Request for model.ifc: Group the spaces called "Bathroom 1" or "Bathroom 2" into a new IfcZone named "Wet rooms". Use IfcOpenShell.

First a look at what the model holds.

```python
import ifcopenshell

model = ifcopenshell.open("model.ifc")
print(model.schema)
seen = {}
for space in model.by_type("IfcSpace"):
    seen[space.LongName] = seen.get(space.LongName, 0) + 1
for name, count in sorted(seen.items(), key=str):
    print(count, "x", name)
print("zones:", [z.Name for z in model.by_type("IfcZone")][:20])
```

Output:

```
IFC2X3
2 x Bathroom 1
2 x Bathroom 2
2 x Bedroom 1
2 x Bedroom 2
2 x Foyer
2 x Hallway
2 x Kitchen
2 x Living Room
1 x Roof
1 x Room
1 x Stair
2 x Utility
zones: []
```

```python
import ifcopenshell
import ifcopenshell.api.group
import ifcopenshell.api.root

model = ifcopenshell.open("model.ifc")

names = {"Bathroom 1", "Bathroom 2"}
spaces = [s for s in model.by_type("IfcSpace") if s.LongName in names]

zone = ifcopenshell.api.root.create_entity(model, ifc_class="IfcZone", name="Wet rooms")
ifcopenshell.api.group.assign_group(model, products=spaces, group=zone)
print(len(spaces), "spaces in", zone.Name)

model.write("model_rev.ifc")
```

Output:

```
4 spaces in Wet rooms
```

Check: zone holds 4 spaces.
